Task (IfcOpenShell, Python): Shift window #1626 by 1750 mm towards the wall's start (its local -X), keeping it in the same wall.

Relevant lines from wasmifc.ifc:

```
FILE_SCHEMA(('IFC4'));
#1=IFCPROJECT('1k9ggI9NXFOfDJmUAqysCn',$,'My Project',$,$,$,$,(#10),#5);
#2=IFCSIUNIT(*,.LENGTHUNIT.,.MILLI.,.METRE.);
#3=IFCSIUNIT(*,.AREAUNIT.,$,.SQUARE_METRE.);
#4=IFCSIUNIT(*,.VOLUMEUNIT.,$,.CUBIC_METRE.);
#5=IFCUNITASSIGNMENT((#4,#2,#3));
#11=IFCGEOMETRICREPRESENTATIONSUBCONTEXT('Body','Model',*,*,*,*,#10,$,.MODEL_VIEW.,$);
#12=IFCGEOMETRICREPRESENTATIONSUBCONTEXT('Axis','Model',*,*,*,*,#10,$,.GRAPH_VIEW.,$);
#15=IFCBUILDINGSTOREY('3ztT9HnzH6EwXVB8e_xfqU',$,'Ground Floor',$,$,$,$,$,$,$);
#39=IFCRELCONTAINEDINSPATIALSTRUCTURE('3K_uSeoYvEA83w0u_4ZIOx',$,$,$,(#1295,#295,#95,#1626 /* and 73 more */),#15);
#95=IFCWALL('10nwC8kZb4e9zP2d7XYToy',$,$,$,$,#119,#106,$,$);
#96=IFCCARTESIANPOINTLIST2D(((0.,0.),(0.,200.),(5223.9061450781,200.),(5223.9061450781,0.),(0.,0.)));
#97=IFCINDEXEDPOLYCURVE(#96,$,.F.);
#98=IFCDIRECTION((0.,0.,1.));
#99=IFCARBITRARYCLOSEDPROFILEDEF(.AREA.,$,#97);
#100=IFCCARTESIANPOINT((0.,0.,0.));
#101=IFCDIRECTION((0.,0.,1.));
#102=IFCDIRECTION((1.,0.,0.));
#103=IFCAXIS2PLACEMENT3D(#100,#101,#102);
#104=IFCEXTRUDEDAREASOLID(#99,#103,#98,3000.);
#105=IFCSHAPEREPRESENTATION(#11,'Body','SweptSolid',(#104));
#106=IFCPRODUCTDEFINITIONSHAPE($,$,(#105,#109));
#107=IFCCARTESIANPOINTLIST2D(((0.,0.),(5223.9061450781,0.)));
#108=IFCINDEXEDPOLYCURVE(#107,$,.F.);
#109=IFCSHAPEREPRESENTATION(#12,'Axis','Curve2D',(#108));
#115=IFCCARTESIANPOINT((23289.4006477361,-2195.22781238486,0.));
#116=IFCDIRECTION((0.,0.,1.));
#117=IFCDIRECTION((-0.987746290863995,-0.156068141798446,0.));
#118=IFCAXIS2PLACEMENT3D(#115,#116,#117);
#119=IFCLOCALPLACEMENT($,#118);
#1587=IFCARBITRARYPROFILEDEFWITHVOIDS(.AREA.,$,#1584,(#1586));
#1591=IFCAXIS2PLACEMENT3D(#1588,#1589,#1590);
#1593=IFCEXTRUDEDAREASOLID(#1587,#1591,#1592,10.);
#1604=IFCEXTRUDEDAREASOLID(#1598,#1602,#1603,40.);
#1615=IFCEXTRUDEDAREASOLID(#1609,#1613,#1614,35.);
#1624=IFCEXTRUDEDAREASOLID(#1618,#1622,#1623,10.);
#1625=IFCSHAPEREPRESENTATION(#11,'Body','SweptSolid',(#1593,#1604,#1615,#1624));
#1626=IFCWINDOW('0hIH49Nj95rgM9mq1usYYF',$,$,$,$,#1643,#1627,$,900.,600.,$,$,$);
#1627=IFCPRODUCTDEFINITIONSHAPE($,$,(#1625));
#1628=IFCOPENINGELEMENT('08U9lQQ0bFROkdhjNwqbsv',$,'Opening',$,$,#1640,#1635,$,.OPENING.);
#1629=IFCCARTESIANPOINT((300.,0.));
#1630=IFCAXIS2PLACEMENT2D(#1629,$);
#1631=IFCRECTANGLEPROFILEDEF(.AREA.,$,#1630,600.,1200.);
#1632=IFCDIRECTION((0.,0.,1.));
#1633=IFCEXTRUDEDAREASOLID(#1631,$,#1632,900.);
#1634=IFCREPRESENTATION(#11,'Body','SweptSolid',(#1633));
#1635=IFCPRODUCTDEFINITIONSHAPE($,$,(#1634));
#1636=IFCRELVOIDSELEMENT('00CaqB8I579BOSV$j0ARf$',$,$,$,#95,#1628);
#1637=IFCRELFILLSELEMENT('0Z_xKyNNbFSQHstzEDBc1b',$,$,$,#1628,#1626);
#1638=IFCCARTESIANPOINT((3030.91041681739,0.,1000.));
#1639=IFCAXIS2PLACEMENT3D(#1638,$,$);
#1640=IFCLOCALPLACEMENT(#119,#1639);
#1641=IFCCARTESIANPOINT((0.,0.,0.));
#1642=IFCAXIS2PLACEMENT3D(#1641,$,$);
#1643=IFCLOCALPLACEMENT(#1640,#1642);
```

```python
import ifcopenshell
import ifcopenshell.api.geometry
import ifcopenshell.util.placement

model = ifcopenshell.open("wasmifc.ifc")

window = model.by_guid("0hIH49Nj95rgM9mq1usYYF")
opening = window.FillsVoids[0].RelatingOpeningElement
wall = opening.VoidsElements[0].RelatingBuildingElement

wall_matrix = ifcopenshell.util.placement.get_local_placement(wall.ObjectPlacement)
shift = wall_matrix[:3, 0] * -1750.0
before = ifcopenshell.util.placement.get_local_placement(window.ObjectPlacement)[:3, 3].copy()

# The window is placed relative to its opening, so it follows when the opening moves.
matrix = ifcopenshell.util.placement.get_local_placement(opening.ObjectPlacement)
matrix[:3, 3] += shift
ifcopenshell.api.geometry.edit_object_placement(
    model, product=opening, matrix=matrix, is_si=False, should_transform_children=True
)

after = ifcopenshell.util.placement.get_local_placement(window.ObjectPlacement)[:3, 3]
print("window moved by", (after - before).round(3) + 0.0)

model.write("wasmifc_edited.ifc")
```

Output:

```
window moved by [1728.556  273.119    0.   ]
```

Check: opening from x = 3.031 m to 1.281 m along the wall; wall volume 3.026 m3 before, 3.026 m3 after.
